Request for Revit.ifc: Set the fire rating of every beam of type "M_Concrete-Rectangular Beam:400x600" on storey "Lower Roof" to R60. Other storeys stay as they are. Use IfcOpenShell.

First a look at what the model holds.

```python
import ifcopenshell
import ifcopenshell.util.element

model = ifcopenshell.open("Revit.ifc")
print(model.schema)
storey = next(s for s in model.by_type("IfcBuildingStorey") if s.Name == "Lower Roof")
beams = [e for e in ifcopenshell.util.element.get_decomposition(storey) if e.is_a("IfcBeam")]
seen = {}
for e in beams:
    element_type = ifcopenshell.util.element.get_type(e)
    key = (element_type.Name if element_type != e and element_type else None, ifcopenshell.util.element.get_pset(e, "Pset_BeamCommon", "FireRating"))
    seen[key] = seen.get(key, 0) + 1
for (name, value), count in sorted(seen.items(), key=str):
    print(count, "x", name, "|", value)
```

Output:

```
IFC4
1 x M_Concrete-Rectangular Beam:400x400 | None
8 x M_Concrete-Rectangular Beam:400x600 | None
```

```python
import ifcopenshell
import ifcopenshell.api.pset
import ifcopenshell.util.element

model = ifcopenshell.open("Revit.ifc")

storey = next(s for s in model.by_type("IfcBuildingStorey") if s.Name == "Lower Roof")
beams = [e for e in ifcopenshell.util.element.get_decomposition(storey) if e.is_a("IfcBeam")]

count = 0
for e in beams:
    element_type = ifcopenshell.util.element.get_type(e)
    if element_type in (None, e) or element_type.Name != "M_Concrete-Rectangular Beam:400x600":
        continue
    # add_pset returns the element's existing set when there is one.
    pset = ifcopenshell.api.pset.add_pset(model, product=e, name="Pset_BeamCommon")
    ifcopenshell.api.pset.edit_pset(model, pset=pset, properties={"FireRating": "R60"})
    count += 1

print(count, "beams updated")

model.write("Revit-out.ifc")
```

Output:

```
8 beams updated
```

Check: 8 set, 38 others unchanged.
